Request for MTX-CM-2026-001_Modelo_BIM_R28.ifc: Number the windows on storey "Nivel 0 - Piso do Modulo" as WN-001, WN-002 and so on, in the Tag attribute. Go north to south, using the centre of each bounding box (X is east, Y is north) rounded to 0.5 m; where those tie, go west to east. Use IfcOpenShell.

First a look at what the model holds.

```python
import ifcopenshell
import ifcopenshell.util.element
import ifcopenshell.util.placement

model = ifcopenshell.open("MTX-CM-2026-001_Modelo_BIM_R28.ifc")
print(model.schema)
storey = next(s for s in model.by_type("IfcBuildingStorey") if s.Name == "Nivel 0 - Piso do Modulo")
windows = [e for e in ifcopenshell.util.element.get_decomposition(storey) if e.is_a("IfcWindow")]
for e in sorted(windows, key=lambda e: e.id()):
    origin = ifcopenshell.util.placement.get_local_placement(e.ObjectPlacement)[:3, 3]
    print(e.id(), e.Tag, e.Name, origin.round(2) + 0.0, sep=" | ")
```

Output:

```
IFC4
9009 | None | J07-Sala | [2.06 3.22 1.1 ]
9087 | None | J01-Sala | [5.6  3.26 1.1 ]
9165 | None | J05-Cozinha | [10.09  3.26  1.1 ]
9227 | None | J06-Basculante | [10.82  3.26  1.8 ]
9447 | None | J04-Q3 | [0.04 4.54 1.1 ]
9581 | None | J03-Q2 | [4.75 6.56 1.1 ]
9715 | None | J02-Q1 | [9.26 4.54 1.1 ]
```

```python
import ifcopenshell
import ifcopenshell.geom
import ifcopenshell.util.element
import ifcopenshell.util.shape

model = ifcopenshell.open("MTX-CM-2026-001_Modelo_BIM_R28.ifc")
settings = ifcopenshell.geom.settings()
settings.set("use-world-coords", True)


def centre(element):
    shape = ifcopenshell.geom.create_shape(settings, element)
    return ifcopenshell.util.shape.get_bbox_centroid(shape.geometry)


storey = next(s for s in model.by_type("IfcBuildingStorey") if s.Name == "Nivel 0 - Piso do Modulo")
windows = [e for e in ifcopenshell.util.element.get_decomposition(storey) if e.is_a("IfcWindow")]

# Insertion points can sit at a corner or the storey origin, so sort by the geometry (in metres).
centres = {e: centre(e) for e in windows}
windows.sort(key=lambda e: (-round(centres[e][1] / 0.5), centres[e][0]))

for i, e in enumerate(windows, start=1):
    number = f"WN-0{i:02d}"
    e.Tag = number
    print(e.id(), number)

model.write("MTX-CM-2026-001_Modelo_BIM_R28_rev.ifc")
```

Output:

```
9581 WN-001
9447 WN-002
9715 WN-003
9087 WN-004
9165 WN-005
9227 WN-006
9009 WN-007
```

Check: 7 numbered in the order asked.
